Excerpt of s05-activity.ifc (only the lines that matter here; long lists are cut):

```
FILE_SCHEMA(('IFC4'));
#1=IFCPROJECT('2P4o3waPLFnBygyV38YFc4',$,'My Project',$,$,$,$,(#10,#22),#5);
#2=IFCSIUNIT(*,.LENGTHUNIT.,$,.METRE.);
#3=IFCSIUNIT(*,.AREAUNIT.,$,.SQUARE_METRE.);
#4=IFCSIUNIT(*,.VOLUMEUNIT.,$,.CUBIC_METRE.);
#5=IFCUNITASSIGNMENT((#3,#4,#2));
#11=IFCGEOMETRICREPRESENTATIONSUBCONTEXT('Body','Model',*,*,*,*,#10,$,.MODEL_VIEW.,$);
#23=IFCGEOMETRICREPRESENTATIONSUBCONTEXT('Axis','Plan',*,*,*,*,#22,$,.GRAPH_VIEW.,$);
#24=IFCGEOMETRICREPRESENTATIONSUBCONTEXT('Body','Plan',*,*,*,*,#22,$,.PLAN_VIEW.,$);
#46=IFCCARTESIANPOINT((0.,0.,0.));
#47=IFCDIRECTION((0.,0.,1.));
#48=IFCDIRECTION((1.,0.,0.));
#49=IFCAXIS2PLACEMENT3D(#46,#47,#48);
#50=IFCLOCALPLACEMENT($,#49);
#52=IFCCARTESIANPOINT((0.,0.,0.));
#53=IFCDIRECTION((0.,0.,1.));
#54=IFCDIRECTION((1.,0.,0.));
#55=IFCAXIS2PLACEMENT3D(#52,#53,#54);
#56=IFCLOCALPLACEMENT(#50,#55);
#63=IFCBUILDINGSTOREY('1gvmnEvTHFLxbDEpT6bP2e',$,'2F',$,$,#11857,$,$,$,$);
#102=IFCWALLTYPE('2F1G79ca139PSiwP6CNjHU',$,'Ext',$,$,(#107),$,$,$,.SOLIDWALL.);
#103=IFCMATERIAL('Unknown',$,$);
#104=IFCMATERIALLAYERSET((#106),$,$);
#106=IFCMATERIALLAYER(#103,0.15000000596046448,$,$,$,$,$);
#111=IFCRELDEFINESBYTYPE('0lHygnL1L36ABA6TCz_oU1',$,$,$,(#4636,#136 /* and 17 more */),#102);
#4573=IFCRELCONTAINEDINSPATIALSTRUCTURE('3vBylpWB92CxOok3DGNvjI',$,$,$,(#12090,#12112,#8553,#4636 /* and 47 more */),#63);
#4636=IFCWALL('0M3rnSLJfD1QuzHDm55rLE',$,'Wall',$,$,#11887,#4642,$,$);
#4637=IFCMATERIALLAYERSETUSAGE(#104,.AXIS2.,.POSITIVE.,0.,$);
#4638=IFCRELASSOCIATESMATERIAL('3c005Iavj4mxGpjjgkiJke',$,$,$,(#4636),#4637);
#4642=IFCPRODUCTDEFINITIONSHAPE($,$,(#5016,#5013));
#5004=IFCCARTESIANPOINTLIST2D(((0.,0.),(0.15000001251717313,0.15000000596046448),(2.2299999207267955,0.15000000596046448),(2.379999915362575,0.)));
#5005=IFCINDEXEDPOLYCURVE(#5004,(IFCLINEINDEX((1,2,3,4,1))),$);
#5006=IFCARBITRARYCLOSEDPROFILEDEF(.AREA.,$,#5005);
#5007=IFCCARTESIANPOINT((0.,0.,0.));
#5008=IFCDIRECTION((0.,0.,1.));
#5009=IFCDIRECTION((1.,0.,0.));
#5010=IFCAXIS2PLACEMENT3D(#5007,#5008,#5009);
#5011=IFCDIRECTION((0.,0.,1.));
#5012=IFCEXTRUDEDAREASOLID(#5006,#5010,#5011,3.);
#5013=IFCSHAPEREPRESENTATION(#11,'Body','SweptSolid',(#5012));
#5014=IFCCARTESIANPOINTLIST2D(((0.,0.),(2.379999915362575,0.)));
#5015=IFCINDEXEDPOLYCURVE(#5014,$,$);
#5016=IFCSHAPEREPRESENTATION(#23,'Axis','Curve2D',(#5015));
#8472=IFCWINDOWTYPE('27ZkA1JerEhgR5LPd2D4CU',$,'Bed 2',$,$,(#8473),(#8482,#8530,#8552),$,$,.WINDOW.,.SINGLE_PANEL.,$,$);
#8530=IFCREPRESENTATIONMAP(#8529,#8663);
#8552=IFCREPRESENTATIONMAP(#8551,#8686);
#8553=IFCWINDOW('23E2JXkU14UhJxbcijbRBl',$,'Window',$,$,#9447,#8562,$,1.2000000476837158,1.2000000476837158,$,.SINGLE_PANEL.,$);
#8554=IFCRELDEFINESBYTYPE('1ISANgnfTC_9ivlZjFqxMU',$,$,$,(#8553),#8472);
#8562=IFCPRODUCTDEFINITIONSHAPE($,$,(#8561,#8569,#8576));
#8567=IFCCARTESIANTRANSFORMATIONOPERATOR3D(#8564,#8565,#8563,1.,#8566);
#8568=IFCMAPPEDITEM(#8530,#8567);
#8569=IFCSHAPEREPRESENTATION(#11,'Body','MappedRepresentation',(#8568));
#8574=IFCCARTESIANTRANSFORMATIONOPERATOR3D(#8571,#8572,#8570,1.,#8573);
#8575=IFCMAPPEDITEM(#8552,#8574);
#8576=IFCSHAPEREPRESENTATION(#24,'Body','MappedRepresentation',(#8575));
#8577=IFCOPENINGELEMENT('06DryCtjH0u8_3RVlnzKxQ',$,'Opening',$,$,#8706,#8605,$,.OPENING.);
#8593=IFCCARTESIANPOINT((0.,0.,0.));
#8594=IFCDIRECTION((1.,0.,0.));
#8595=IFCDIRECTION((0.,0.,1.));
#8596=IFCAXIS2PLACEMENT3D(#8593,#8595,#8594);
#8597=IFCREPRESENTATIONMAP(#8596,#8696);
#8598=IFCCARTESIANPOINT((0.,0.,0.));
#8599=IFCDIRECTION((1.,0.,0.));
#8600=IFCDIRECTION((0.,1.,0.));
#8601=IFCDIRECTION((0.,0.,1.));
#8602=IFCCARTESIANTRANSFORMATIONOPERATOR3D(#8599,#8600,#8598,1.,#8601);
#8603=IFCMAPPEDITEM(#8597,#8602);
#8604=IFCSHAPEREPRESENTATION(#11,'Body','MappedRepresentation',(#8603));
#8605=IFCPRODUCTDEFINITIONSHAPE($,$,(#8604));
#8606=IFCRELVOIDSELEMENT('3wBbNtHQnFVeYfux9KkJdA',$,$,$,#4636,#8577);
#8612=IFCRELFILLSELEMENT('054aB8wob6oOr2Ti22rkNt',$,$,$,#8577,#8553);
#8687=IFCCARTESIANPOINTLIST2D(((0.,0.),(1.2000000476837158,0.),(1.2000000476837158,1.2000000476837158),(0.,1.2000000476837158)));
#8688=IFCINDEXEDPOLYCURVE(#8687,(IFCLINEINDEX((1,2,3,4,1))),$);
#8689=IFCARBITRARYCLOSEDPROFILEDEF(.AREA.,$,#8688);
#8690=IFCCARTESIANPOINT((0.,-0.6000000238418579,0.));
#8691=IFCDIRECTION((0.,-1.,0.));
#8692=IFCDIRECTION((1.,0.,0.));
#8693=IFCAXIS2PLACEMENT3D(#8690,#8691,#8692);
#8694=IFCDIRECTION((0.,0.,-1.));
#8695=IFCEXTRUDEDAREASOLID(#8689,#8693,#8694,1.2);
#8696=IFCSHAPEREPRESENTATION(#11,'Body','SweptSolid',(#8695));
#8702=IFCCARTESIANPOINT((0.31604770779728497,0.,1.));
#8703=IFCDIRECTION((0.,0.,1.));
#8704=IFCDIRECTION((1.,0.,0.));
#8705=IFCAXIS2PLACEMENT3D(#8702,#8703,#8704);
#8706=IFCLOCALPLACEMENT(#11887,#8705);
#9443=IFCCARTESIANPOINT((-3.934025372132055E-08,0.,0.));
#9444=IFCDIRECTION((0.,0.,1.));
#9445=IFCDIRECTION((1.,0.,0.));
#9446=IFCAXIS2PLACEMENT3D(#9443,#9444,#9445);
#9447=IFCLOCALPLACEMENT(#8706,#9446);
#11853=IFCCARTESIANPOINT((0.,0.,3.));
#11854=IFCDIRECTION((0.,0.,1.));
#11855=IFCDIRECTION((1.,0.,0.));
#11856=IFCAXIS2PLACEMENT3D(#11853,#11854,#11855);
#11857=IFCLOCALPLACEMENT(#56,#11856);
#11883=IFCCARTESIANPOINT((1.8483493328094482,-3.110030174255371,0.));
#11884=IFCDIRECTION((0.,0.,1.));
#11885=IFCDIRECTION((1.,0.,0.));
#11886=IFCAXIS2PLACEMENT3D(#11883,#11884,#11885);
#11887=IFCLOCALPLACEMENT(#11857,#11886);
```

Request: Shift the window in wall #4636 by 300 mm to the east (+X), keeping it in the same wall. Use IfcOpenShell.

```python
import ifcopenshell
import ifcopenshell.api.geometry
import ifcopenshell.util.placement

model = ifcopenshell.open("s05-activity.ifc")

window = model.by_id(8553)
opening = window.FillsVoids[0].RelatingOpeningElement
wall = opening.VoidsElements[0].RelatingBuildingElement

wall_matrix = ifcopenshell.util.placement.get_local_placement(wall.ObjectPlacement)
shift = wall_matrix[:3, 0] * 0.3
before = ifcopenshell.util.placement.get_local_placement(window.ObjectPlacement)[:3, 3].copy()

# The window is placed relative to its opening, so it follows when the opening moves.
matrix = ifcopenshell.util.placement.get_local_placement(opening.ObjectPlacement)
matrix[:3, 3] += shift
ifcopenshell.api.geometry.edit_object_placement(
    model, product=opening, matrix=matrix, is_si=False, should_transform_children=True
)

after = ifcopenshell.util.placement.get_local_placement(window.ObjectPlacement)[:3, 3]
print("window moved by", (after - before).round(3) + 0.0)

model.write("s05-activity_v2.ifc")
```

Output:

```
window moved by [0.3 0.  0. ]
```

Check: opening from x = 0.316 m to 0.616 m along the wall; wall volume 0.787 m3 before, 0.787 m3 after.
